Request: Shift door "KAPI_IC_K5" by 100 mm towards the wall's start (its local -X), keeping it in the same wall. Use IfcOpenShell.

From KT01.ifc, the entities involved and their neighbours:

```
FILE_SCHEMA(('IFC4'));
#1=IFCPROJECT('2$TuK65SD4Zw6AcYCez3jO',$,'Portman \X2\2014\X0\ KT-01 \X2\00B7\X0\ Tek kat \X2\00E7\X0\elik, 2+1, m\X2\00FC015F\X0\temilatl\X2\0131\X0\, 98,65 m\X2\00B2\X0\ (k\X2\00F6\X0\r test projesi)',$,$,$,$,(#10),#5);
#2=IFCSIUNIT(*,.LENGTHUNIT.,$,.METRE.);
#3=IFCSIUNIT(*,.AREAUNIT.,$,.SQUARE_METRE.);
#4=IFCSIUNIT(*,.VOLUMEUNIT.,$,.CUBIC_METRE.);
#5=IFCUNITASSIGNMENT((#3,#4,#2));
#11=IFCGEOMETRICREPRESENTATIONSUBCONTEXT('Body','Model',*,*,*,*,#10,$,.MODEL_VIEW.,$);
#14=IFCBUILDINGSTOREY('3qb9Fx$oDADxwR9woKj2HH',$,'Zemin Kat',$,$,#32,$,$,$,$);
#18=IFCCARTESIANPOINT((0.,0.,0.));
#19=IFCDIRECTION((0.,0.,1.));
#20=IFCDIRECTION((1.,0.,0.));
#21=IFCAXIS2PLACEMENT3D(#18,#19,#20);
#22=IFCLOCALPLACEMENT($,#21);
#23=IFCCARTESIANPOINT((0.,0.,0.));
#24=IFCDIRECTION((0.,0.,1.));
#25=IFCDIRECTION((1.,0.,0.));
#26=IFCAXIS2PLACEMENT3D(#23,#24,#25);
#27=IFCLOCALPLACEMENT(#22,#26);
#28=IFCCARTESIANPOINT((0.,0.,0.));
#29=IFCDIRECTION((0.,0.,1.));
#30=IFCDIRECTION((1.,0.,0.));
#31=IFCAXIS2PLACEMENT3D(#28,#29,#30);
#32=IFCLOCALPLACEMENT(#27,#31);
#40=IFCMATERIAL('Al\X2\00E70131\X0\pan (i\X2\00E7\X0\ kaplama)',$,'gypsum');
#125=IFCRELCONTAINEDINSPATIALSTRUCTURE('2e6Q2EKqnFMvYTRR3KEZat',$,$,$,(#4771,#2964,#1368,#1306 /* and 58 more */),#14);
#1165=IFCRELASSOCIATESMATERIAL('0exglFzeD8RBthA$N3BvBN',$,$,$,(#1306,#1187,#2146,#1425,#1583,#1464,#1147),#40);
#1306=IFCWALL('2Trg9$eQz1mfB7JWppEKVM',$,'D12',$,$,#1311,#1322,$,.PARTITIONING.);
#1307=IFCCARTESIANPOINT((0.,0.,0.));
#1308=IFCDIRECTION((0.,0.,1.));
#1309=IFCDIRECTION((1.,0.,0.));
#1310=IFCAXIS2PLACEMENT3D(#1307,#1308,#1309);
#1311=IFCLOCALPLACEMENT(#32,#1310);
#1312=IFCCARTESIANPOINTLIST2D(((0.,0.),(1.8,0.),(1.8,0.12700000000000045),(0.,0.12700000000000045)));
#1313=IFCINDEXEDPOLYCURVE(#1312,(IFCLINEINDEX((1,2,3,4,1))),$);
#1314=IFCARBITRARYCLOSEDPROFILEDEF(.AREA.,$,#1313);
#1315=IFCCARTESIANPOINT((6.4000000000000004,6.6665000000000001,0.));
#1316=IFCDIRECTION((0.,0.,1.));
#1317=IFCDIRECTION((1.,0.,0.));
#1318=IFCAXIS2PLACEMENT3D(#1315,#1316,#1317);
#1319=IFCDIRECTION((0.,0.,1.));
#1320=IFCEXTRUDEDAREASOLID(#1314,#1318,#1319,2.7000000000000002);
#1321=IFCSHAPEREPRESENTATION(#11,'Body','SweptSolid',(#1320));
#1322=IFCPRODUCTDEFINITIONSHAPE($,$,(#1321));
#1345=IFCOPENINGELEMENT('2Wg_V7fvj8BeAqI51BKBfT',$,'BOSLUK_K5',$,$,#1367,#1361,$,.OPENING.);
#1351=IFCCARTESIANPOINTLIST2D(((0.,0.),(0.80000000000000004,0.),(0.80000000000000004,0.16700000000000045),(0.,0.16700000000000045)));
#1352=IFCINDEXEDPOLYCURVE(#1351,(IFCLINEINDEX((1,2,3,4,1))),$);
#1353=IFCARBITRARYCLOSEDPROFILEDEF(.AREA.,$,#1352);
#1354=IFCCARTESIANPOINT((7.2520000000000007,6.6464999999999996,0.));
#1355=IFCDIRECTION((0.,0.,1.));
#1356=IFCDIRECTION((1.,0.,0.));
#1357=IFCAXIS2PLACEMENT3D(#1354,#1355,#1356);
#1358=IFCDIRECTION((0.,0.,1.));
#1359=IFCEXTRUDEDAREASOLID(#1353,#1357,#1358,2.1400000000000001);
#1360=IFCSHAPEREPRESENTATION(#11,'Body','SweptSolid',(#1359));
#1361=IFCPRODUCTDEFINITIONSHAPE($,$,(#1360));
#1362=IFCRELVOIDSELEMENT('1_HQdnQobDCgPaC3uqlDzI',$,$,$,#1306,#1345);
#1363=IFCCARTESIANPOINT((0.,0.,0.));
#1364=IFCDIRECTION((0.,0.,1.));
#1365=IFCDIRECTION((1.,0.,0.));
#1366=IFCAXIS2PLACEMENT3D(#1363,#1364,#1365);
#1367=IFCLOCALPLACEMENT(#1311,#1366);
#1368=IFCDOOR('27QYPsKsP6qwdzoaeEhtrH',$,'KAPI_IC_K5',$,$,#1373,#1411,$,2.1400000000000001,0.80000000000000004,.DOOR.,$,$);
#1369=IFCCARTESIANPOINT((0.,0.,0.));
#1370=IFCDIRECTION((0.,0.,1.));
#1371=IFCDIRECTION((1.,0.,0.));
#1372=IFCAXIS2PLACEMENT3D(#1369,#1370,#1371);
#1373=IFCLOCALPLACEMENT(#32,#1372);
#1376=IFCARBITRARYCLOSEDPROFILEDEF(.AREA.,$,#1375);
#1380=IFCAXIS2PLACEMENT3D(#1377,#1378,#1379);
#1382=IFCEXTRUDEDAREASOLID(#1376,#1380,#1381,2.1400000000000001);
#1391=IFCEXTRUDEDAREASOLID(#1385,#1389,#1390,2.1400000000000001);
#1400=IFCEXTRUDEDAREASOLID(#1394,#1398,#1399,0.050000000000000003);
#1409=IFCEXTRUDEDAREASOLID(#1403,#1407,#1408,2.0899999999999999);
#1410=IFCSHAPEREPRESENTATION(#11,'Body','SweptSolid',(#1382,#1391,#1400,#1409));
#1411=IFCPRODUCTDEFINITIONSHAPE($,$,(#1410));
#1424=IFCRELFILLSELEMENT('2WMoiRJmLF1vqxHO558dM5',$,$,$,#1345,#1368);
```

```python
import ifcopenshell
import ifcopenshell.api.geometry
import ifcopenshell.util.placement

model = ifcopenshell.open("KT01.ifc")

door = model.by_id(1368)
opening = door.FillsVoids[0].RelatingOpeningElement
wall = opening.VoidsElements[0].RelatingBuildingElement

wall_matrix = ifcopenshell.util.placement.get_local_placement(wall.ObjectPlacement)
shift = wall_matrix[:3, 0] * -0.1
before = ifcopenshell.util.placement.get_local_placement(door.ObjectPlacement)[:3, 3].copy()

# The door is not placed relative to its opening, so move both.
for product in (opening, door):
    matrix = ifcopenshell.util.placement.get_local_placement(product.ObjectPlacement)
    matrix[:3, 3] += shift
    ifcopenshell.api.geometry.edit_object_placement(model, product=product, matrix=matrix, is_si=False)

after = ifcopenshell.util.placement.get_local_placement(door.ObjectPlacement)[:3, 3]
print("door moved by", (after - before).round(3) + 0.0)

model.write("KT01-out.ifc")
```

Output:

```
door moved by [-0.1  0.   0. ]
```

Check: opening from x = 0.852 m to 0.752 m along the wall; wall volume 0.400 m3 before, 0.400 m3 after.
